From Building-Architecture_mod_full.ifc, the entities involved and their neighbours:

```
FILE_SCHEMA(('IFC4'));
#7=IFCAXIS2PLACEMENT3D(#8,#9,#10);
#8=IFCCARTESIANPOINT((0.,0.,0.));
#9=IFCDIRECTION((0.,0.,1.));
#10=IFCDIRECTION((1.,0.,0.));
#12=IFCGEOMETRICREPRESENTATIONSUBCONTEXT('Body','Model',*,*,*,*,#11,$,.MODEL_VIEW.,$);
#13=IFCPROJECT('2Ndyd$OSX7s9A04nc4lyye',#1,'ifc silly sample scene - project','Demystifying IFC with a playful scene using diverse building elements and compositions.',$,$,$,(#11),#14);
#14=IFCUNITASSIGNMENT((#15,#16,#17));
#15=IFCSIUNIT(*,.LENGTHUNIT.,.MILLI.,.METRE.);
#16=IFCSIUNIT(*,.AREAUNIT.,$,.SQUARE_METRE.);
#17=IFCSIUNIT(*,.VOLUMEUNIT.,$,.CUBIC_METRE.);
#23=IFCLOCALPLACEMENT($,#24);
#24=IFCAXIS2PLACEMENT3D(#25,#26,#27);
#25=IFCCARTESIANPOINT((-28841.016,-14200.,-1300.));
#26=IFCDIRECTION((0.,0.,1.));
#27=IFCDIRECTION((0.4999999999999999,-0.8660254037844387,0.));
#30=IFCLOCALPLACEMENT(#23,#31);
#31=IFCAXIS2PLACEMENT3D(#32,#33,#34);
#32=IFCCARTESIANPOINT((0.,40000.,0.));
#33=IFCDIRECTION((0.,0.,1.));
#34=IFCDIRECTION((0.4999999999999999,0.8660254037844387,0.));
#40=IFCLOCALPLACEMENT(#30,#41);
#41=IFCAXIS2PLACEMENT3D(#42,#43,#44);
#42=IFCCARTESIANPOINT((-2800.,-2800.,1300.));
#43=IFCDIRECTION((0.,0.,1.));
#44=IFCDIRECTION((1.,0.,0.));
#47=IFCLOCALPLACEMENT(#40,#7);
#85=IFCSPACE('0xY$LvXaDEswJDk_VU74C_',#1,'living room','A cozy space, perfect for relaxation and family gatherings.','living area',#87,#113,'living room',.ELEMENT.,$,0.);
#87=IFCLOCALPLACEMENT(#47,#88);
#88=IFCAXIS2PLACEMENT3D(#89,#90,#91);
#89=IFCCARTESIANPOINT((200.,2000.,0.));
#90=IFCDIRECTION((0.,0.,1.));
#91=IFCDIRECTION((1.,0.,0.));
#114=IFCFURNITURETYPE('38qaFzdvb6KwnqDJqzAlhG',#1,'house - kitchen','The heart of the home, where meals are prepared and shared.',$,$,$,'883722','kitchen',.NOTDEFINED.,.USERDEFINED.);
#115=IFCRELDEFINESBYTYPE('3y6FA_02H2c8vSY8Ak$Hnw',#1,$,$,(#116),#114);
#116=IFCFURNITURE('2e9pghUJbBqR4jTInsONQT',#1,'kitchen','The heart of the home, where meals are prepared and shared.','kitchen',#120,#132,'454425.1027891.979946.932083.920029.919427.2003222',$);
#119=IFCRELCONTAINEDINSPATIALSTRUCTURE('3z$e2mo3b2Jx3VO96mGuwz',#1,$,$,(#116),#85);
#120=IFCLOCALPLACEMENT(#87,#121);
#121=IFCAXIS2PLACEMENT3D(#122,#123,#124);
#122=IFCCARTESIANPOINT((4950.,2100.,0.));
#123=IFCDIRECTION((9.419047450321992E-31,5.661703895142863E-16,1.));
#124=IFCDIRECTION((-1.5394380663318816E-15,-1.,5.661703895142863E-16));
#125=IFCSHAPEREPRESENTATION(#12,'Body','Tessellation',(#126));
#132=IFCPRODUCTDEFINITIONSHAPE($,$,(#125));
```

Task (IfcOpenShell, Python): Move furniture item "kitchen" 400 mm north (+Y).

```python
import ifcopenshell
import ifcopenshell.api.geometry
import ifcopenshell.util.placement
import ifcopenshell.util.unit

model = ifcopenshell.open("Building-Architecture_mod_full.ifc")
unit_scale = ifcopenshell.util.unit.calculate_unit_scale(model)

item = model.by_guid("2e9pghUJbBqR4jTInsONQT")
matrix = ifcopenshell.util.placement.get_local_placement(item.ObjectPlacement)
matrix[1, 3] += 0.4 / unit_scale
ifcopenshell.api.geometry.edit_object_placement(model, product=item, matrix=matrix, is_si=False)

print(ifcopenshell.util.placement.get_local_placement(item.ObjectPlacement).round(3) + 0.0)

model.write("Building-Architecture_mod_full_edited.ifc")
```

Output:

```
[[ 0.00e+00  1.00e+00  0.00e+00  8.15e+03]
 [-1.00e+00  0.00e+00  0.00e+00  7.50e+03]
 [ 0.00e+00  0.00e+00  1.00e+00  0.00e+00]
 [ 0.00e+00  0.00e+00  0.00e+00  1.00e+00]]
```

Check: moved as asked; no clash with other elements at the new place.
